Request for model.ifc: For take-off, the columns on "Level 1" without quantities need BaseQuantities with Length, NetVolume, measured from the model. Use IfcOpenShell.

First a look at what the model holds.

```python
import ifcopenshell
import ifcopenshell.util.element
import ifcopenshell.util.unit

model = ifcopenshell.open("model.ifc")
print(model.schema)
for unit_type in ("LENGTHUNIT", "AREAUNIT", "VOLUMEUNIT"):
    print(unit_type, ifcopenshell.util.unit.calculate_unit_scale(model, unit_type))
storey = next(s for s in model.by_type("IfcBuildingStorey") if s.Name == "Level 1")
columns = [e for e in ifcopenshell.util.element.get_decomposition(storey) if e.is_a("IfcColumn")]
for e in sorted(columns, key=lambda e: e.id()):
    print(e.id(), e.is_a(), e.Name, list(ifcopenshell.util.element.get_psets(e, qtos_only=True)), sep=" | ")
```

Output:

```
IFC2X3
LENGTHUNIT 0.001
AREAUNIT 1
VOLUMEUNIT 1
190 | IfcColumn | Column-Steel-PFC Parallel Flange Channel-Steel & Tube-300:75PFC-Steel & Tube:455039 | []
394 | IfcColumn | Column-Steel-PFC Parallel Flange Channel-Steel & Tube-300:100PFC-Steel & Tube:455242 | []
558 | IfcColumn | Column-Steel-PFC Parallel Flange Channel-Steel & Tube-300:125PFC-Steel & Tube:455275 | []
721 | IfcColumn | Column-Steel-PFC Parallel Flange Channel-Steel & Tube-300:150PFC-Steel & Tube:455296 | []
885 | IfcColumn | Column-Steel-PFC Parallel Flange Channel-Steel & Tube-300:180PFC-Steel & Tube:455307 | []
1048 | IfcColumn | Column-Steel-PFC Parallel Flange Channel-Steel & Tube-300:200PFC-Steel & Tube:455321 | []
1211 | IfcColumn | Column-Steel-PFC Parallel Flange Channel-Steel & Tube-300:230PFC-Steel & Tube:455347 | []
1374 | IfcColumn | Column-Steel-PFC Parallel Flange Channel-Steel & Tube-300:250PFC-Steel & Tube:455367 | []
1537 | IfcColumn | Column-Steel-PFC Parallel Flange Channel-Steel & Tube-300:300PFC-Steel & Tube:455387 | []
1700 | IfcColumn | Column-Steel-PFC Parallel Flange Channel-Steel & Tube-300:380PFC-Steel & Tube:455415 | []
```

```python
import ifcopenshell
import ifcopenshell.api.pset
import ifcopenshell.geom
import ifcopenshell.util.element
import ifcopenshell.util.shape
import ifcopenshell.util.unit

model = ifcopenshell.open("model.ifc")
unit_scale = ifcopenshell.util.unit.calculate_unit_scale(model)
volume_scale = ifcopenshell.util.unit.calculate_unit_scale(model, "VOLUMEUNIT")
settings = ifcopenshell.geom.settings()

storey = next(s for s in model.by_type("IfcBuildingStorey") if s.Name == "Level 1")
columns = [e for e in ifcopenshell.util.element.get_decomposition(storey) if e.is_a("IfcColumn")]

for e in sorted(columns, key=lambda e: e.id()):
    if ifcopenshell.util.element.get_psets(e, qtos_only=True, should_inherit=False):
        continue
    # Geometry comes back in metres, in the element's own axes.
    shape = ifcopenshell.geom.create_shape(settings, e)
    values = {
        "Length": ifcopenshell.util.shape.get_z(shape.geometry) / unit_scale,
        "NetVolume": ifcopenshell.util.shape.get_volume(shape.geometry) / volume_scale,
    }
    qto = ifcopenshell.api.pset.add_qto(model, product=e, name="BaseQuantities")
    ifcopenshell.api.pset.edit_qto(model, qto=qto, properties=values)
    print(e.id(), {k: round(v, 3) for k, v in values.items()})

model.write("model_v2.ifc")
```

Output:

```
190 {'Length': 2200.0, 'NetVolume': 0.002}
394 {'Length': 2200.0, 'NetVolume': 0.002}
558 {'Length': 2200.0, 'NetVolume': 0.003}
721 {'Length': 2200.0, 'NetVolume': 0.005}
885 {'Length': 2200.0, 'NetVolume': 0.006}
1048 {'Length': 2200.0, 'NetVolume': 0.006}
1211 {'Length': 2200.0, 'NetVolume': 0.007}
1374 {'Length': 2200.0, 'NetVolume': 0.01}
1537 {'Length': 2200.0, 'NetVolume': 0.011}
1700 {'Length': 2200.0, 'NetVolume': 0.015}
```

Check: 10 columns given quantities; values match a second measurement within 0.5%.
